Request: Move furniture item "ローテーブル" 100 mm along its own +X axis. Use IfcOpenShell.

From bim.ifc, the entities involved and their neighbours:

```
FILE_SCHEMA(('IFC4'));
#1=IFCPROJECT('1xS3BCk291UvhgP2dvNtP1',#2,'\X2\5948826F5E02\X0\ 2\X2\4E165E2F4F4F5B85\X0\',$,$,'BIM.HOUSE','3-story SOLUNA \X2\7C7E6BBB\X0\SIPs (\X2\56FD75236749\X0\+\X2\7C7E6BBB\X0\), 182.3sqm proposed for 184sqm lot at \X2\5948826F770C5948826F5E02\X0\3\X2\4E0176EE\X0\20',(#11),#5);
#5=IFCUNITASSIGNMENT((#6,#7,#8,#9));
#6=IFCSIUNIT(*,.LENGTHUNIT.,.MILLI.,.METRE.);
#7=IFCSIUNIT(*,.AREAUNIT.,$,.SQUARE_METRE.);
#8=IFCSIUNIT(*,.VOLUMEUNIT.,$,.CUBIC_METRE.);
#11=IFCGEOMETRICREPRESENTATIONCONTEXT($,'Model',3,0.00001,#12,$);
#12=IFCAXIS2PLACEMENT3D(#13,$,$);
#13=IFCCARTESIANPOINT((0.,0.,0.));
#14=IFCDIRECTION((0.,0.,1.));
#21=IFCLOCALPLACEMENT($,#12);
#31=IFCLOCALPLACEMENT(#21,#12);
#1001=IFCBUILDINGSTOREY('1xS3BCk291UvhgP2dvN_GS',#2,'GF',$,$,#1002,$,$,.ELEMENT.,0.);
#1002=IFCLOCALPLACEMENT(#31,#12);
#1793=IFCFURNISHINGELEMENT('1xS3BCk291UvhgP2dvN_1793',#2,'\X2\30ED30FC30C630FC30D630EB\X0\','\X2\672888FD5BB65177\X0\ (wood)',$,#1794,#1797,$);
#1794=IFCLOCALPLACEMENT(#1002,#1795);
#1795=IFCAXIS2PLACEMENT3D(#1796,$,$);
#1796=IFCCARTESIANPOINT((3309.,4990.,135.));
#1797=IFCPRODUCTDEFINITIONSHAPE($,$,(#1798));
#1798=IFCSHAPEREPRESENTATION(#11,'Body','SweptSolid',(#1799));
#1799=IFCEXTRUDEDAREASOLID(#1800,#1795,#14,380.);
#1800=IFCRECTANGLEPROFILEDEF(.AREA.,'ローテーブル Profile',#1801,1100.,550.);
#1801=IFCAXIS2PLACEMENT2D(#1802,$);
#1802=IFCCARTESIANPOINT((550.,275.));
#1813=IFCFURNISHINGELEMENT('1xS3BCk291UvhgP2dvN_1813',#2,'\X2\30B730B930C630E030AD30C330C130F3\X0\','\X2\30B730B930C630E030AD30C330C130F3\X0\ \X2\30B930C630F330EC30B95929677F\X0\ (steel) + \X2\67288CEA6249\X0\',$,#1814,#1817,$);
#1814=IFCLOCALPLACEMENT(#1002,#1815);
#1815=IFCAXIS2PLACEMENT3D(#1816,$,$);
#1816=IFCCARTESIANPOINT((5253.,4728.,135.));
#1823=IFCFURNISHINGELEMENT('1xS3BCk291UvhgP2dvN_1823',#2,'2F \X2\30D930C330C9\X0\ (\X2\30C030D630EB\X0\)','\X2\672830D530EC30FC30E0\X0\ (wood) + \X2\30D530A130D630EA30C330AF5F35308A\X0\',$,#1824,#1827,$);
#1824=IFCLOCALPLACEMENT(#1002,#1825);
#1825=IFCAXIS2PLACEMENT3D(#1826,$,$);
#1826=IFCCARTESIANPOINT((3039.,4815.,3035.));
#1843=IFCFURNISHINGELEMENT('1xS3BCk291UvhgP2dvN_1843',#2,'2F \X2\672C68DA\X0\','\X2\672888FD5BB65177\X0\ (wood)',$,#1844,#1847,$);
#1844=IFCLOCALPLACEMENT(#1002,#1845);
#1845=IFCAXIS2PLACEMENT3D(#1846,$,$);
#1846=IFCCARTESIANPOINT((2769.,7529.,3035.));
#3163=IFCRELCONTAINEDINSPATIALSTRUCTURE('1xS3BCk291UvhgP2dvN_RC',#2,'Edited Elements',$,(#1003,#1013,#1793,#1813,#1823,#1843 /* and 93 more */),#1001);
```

```python
import ifcopenshell
import ifcopenshell.api.geometry
import ifcopenshell.util.placement
import ifcopenshell.util.unit

model = ifcopenshell.open("bim.ifc")
unit_scale = ifcopenshell.util.unit.calculate_unit_scale(model)

item = model.by_guid("1xS3BCk291UvhgP2dvN_1793")
matrix = ifcopenshell.util.placement.get_local_placement(item.ObjectPlacement)
matrix[:3, 3] += matrix[:3, 0] * 0.1 / unit_scale
ifcopenshell.api.geometry.edit_object_placement(model, product=item, matrix=matrix, is_si=False)

print(ifcopenshell.util.placement.get_local_placement(item.ObjectPlacement).round(3) + 0.0)

model.write("bim_rev.ifc")
```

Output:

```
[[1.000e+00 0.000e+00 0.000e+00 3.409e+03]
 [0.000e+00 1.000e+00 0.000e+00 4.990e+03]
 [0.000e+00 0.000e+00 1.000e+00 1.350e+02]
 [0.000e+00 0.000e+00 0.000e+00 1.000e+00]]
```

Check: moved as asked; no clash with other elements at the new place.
